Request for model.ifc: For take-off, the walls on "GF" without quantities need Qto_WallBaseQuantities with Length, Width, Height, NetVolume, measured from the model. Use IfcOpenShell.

First a look at what the model holds.

```python
import ifcopenshell
import ifcopenshell.util.element
import ifcopenshell.util.unit

model = ifcopenshell.open("model.ifc")
print(model.schema)
for unit_type in ("LENGTHUNIT", "AREAUNIT", "VOLUMEUNIT"):
    print(unit_type, ifcopenshell.util.unit.calculate_unit_scale(model, unit_type))
storey = next(s for s in model.by_type("IfcBuildingStorey") if s.Name == "GF")
walls = [e for e in ifcopenshell.util.element.get_decomposition(storey) if e.is_a("IfcWall")]
for e in sorted(walls, key=lambda e: e.id()):
    print(e.id(), e.is_a(), e.Name, list(ifcopenshell.util.element.get_psets(e, qtos_only=True)), sep=" | ")
```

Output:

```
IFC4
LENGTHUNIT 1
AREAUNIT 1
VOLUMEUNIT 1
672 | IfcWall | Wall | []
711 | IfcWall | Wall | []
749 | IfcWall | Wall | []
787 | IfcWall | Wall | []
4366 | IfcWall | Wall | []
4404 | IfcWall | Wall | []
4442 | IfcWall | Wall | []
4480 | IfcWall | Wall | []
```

```python
import ifcopenshell
import ifcopenshell.api.pset
import ifcopenshell.geom
import ifcopenshell.util.element
import ifcopenshell.util.shape
import ifcopenshell.util.unit

model = ifcopenshell.open("model.ifc")
unit_scale = ifcopenshell.util.unit.calculate_unit_scale(model)
volume_scale = ifcopenshell.util.unit.calculate_unit_scale(model, "VOLUMEUNIT")
settings = ifcopenshell.geom.settings()

storey = next(s for s in model.by_type("IfcBuildingStorey") if s.Name == "GF")
walls = [e for e in ifcopenshell.util.element.get_decomposition(storey) if e.is_a("IfcWall")]

for e in sorted(walls, key=lambda e: e.id()):
    if ifcopenshell.util.element.get_psets(e, qtos_only=True, should_inherit=False):
        continue
    # Geometry comes back in metres, in the element's own axes.
    shape = ifcopenshell.geom.create_shape(settings, e)
    values = {
        "Length": ifcopenshell.util.shape.get_x(shape.geometry) / unit_scale,
        "Width": ifcopenshell.util.shape.get_y(shape.geometry) / unit_scale,
        "Height": ifcopenshell.util.shape.get_z(shape.geometry) / unit_scale,
        "NetVolume": ifcopenshell.util.shape.get_volume(shape.geometry) / volume_scale,
    }
    qto = ifcopenshell.api.pset.add_qto(model, product=e, name="Qto_WallBaseQuantities")
    ifcopenshell.api.pset.edit_qto(model, qto=qto, properties=values)
    print(e.id(), {k: round(v, 3) for k, v in values.items()})

model.write("model_updated.ifc")
```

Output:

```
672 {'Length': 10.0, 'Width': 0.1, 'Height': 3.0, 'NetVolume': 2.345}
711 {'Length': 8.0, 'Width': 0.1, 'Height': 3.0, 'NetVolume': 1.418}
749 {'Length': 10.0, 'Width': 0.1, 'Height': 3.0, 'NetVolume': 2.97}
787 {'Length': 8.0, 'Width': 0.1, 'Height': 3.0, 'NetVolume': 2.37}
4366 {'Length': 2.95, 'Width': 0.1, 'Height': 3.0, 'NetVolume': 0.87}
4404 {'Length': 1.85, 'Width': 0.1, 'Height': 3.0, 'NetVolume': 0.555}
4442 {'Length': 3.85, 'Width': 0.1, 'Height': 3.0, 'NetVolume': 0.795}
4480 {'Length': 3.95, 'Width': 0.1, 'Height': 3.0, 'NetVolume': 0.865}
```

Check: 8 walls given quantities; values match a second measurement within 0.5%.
